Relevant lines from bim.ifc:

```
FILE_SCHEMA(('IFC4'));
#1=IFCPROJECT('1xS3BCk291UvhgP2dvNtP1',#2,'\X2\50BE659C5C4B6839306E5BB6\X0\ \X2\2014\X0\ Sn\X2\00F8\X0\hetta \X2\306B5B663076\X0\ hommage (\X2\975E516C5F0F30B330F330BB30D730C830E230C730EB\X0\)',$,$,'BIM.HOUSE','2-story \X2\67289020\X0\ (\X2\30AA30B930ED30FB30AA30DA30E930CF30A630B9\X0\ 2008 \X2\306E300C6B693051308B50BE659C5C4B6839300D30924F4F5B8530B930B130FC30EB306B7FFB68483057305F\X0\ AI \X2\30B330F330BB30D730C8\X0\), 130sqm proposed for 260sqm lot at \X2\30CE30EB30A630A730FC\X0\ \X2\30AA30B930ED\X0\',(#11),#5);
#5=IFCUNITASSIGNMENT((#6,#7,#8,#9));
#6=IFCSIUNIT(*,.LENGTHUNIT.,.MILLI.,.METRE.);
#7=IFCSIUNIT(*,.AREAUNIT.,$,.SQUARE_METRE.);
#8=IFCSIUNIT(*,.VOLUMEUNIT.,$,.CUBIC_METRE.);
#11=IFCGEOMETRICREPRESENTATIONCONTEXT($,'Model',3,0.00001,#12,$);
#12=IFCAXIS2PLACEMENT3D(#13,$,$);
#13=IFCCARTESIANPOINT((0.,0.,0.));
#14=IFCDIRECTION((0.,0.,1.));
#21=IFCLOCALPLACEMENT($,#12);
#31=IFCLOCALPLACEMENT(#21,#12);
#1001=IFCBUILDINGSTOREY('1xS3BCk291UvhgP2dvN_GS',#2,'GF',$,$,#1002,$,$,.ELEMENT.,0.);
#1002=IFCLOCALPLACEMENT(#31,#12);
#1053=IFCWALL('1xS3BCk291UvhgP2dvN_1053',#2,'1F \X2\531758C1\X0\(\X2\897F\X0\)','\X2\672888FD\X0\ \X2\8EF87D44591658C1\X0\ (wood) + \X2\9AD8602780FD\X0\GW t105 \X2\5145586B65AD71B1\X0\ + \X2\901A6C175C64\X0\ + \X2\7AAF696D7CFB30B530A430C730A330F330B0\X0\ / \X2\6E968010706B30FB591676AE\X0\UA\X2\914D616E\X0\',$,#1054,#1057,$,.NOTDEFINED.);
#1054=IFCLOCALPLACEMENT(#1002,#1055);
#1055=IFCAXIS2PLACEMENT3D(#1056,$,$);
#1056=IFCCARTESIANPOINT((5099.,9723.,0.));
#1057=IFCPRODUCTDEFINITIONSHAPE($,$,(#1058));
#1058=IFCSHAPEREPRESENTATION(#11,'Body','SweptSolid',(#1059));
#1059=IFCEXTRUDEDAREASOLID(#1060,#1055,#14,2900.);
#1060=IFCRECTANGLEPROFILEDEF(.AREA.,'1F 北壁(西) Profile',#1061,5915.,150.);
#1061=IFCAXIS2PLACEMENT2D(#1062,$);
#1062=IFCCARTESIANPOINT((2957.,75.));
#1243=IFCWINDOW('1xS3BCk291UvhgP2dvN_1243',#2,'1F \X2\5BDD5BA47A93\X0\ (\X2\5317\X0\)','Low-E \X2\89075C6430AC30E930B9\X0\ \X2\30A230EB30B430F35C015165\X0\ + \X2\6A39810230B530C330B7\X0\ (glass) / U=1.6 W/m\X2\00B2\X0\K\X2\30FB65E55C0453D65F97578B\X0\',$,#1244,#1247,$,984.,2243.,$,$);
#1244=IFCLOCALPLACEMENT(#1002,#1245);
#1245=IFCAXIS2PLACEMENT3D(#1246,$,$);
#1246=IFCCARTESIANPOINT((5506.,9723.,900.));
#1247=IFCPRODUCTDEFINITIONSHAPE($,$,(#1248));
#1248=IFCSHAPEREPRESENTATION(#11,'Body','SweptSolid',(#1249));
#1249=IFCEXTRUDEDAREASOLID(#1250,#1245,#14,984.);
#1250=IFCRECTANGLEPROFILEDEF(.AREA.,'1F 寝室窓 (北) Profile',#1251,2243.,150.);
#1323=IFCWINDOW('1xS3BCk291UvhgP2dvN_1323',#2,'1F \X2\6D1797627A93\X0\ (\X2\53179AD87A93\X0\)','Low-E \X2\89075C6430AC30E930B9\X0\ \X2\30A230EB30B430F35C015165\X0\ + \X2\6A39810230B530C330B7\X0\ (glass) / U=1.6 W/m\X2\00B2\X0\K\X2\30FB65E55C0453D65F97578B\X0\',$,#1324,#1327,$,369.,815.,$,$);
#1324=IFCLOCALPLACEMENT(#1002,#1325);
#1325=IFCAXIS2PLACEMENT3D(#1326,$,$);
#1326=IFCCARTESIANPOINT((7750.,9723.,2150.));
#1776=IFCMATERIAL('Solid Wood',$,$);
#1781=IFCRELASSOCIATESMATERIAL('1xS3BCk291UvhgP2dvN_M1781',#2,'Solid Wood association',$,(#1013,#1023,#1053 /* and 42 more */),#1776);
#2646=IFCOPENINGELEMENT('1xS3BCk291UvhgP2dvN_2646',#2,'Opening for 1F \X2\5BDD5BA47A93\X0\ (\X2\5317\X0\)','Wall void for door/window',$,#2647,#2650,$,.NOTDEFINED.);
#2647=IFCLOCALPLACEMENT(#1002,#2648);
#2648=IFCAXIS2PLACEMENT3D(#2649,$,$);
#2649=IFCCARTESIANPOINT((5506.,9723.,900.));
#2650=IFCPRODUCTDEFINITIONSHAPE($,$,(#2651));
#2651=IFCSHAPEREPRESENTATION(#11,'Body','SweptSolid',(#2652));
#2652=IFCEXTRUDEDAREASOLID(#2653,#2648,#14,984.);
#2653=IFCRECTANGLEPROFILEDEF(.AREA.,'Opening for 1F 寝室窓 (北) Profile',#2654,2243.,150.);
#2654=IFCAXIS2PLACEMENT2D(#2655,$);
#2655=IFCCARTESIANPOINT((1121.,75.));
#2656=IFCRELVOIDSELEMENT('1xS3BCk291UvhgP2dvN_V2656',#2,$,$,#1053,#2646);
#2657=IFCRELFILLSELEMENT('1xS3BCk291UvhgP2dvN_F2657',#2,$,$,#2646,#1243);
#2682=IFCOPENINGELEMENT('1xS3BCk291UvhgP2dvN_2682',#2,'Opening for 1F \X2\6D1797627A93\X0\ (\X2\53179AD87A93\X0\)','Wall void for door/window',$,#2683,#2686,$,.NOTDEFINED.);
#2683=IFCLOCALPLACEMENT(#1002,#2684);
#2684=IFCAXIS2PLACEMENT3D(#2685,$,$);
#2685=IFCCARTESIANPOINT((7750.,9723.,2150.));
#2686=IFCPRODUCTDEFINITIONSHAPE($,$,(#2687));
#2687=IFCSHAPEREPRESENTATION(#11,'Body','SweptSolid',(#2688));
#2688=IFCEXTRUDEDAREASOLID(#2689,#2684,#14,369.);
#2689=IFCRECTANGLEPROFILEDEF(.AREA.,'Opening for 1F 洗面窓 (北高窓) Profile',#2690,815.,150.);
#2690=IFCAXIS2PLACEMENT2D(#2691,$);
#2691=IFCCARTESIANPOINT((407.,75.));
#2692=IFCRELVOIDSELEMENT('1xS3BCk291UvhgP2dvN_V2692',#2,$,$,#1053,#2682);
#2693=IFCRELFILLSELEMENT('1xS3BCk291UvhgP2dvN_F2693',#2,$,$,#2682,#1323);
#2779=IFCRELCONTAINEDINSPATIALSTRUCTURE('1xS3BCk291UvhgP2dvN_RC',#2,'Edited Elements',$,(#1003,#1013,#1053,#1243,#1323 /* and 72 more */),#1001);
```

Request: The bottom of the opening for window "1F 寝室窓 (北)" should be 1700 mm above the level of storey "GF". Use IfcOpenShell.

```python
import numpy as np
import ifcopenshell
import ifcopenshell.api.geometry
import ifcopenshell.geom
import ifcopenshell.util.element
import ifcopenshell.util.placement
import ifcopenshell.util.shape
import ifcopenshell.util.unit

model = ifcopenshell.open("bim.ifc")
unit_scale = ifcopenshell.util.unit.calculate_unit_scale(model)

window = model.by_id(1243)
opening = window.FillsVoids[0].RelatingOpeningElement
storey = ifcopenshell.util.element.get_container(window, ifc_class="IfcBuildingStorey")
level = ifcopenshell.util.placement.get_local_placement(storey.ObjectPlacement)[2, 3]

# The opening's origin need not be at the sill, so measure its lowest point.
shape = ifcopenshell.geom.create_shape(ifcopenshell.geom.settings(), opening)
bottom = ifcopenshell.util.shape.get_shape_bottom_elevation(shape, shape.geometry) / unit_scale
dz = level + 1.7 / unit_scale - bottom

shift = np.array([0.0, 0.0, dz])
# The window is not placed relative to its opening, so move both.
for product in (opening, window):
    matrix = ifcopenshell.util.placement.get_local_placement(product.ObjectPlacement)
    matrix[:3, 3] += shift
    ifcopenshell.api.geometry.edit_object_placement(model, product=product, matrix=matrix, is_si=False)

print(f"moved by {dz * unit_scale:+.3f} m")

model.write("bim_updated.ifc")
```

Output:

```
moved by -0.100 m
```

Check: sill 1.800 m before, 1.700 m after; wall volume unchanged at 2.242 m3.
